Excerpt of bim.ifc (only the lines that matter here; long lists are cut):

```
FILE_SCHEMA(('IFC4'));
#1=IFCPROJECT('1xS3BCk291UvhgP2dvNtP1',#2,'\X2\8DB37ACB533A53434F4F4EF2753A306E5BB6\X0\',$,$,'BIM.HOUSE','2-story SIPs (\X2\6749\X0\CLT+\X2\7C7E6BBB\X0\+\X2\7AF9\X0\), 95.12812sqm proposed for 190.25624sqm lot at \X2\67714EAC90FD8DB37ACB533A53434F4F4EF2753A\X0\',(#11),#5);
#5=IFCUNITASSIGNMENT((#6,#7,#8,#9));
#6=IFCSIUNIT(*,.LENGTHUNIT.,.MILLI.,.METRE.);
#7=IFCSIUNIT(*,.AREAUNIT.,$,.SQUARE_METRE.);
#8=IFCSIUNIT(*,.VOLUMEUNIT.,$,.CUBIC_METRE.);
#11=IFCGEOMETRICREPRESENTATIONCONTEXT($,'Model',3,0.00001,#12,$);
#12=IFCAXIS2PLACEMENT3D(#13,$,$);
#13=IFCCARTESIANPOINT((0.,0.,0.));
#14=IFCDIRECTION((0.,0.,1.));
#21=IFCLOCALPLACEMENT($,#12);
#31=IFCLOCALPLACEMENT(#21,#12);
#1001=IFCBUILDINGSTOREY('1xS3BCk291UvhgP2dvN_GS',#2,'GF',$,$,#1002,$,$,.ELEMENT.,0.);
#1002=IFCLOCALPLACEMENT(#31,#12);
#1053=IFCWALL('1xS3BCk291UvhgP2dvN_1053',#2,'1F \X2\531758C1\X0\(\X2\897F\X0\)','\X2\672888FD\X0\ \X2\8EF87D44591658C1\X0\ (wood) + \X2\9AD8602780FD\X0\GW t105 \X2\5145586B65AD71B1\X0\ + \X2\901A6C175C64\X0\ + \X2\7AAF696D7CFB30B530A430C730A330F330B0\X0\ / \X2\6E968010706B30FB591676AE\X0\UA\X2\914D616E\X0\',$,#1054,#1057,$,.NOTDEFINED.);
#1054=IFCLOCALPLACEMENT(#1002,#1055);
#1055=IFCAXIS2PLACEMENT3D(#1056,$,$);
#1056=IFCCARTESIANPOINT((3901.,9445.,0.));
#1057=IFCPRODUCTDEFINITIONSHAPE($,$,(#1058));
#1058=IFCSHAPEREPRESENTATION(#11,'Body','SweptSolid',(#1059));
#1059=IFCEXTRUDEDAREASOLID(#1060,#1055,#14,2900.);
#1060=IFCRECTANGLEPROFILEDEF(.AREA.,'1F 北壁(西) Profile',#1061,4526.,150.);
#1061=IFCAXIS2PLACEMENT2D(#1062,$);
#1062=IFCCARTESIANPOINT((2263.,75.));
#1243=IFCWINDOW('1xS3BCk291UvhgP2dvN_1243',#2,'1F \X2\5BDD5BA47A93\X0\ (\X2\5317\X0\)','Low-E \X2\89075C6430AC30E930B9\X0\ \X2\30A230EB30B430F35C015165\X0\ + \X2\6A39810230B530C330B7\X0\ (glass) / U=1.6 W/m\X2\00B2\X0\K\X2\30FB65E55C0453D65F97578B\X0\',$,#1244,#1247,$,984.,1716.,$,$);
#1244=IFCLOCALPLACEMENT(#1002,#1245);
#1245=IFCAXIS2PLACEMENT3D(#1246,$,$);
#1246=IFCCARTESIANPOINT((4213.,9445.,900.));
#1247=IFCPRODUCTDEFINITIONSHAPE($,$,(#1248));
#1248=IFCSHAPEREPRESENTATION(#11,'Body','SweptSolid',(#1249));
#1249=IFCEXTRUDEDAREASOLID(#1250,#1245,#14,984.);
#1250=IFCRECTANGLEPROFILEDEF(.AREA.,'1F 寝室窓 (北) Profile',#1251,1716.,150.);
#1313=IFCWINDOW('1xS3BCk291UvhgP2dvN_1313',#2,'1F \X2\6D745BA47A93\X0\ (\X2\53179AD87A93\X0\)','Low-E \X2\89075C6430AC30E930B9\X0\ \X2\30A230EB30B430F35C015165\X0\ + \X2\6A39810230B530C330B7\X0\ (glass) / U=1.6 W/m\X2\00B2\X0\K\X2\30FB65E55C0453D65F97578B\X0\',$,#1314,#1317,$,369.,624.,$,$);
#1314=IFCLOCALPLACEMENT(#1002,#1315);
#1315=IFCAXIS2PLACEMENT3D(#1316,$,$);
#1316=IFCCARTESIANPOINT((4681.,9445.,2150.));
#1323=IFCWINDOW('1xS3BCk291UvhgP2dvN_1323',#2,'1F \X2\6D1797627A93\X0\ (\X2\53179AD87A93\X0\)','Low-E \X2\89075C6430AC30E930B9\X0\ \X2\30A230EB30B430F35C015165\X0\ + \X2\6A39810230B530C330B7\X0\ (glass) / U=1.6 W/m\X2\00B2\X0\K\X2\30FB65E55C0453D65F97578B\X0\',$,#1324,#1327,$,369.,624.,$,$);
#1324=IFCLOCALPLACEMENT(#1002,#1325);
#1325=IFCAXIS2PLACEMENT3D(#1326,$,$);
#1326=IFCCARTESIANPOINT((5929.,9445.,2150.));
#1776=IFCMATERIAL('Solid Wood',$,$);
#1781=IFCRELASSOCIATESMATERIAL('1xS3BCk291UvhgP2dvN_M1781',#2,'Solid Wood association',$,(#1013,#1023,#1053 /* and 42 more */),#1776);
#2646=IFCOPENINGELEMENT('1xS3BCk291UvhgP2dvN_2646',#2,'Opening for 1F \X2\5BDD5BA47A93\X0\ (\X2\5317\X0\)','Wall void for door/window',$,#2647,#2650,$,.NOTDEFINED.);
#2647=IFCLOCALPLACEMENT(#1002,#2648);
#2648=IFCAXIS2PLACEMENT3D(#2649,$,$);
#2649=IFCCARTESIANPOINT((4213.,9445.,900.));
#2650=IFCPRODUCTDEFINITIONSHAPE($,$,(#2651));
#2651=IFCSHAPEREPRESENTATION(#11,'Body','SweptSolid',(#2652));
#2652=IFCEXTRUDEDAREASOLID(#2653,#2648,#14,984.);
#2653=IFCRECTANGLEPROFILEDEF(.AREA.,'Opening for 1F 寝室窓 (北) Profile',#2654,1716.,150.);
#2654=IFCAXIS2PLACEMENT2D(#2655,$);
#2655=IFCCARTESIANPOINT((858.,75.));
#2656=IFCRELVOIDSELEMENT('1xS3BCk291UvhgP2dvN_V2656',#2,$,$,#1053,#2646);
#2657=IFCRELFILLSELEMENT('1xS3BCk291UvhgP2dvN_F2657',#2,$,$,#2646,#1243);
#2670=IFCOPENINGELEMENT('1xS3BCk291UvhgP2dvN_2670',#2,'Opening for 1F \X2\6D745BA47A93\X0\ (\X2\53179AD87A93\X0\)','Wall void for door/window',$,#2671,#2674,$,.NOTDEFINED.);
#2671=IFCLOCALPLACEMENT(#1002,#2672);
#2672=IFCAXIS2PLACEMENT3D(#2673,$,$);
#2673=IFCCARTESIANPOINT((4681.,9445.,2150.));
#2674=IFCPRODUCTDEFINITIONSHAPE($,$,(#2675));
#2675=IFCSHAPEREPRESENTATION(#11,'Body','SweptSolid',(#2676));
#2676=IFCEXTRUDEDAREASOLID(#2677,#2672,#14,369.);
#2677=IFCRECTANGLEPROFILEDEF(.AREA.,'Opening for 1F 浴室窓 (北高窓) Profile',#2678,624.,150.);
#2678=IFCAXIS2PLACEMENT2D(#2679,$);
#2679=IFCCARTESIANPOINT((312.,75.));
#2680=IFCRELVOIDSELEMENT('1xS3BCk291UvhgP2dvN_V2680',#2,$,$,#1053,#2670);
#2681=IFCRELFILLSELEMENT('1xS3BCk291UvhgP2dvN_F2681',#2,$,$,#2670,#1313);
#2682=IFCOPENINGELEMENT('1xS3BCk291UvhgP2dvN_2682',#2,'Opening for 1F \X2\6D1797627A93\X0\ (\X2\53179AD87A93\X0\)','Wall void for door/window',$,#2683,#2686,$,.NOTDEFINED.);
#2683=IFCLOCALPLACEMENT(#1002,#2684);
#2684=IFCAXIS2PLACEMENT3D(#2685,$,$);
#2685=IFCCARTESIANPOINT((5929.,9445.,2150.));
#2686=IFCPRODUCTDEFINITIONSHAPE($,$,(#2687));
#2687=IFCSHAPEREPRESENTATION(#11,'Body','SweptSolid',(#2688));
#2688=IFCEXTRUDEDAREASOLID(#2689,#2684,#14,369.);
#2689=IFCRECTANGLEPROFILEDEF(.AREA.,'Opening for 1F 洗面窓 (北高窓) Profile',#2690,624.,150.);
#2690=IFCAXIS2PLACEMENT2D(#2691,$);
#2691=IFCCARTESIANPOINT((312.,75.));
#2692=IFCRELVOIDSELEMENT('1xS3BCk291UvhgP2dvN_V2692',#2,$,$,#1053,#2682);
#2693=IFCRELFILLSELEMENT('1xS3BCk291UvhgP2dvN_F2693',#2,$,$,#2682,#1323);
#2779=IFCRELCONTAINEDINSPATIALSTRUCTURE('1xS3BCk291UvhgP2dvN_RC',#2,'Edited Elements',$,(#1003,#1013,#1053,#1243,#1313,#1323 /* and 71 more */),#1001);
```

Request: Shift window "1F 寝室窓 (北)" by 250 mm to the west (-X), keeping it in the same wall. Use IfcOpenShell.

```python
import ifcopenshell
import ifcopenshell.api.geometry
import ifcopenshell.util.placement
import ifcopenshell.util.unit

model = ifcopenshell.open("bim.ifc")
unit_scale = ifcopenshell.util.unit.calculate_unit_scale(model)

window = model.by_guid("1xS3BCk291UvhgP2dvN_1243")
opening = window.FillsVoids[0].RelatingOpeningElement
wall = opening.VoidsElements[0].RelatingBuildingElement

wall_matrix = ifcopenshell.util.placement.get_local_placement(wall.ObjectPlacement)
shift = wall_matrix[:3, 0] * -0.25 / unit_scale
before = ifcopenshell.util.placement.get_local_placement(window.ObjectPlacement)[:3, 3].copy()

# The window is not placed relative to its opening, so move both.
for product in (opening, window):
    matrix = ifcopenshell.util.placement.get_local_placement(product.ObjectPlacement)
    matrix[:3, 3] += shift
    ifcopenshell.api.geometry.edit_object_placement(model, product=product, matrix=matrix, is_si=False)

after = ifcopenshell.util.placement.get_local_placement(window.ObjectPlacement)[:3, 3]
print("window moved by", (after - before).round(3) + 0.0)

model.write("bim_v2.ifc")
```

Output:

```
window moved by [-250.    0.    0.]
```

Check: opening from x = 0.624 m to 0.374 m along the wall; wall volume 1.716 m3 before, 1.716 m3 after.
